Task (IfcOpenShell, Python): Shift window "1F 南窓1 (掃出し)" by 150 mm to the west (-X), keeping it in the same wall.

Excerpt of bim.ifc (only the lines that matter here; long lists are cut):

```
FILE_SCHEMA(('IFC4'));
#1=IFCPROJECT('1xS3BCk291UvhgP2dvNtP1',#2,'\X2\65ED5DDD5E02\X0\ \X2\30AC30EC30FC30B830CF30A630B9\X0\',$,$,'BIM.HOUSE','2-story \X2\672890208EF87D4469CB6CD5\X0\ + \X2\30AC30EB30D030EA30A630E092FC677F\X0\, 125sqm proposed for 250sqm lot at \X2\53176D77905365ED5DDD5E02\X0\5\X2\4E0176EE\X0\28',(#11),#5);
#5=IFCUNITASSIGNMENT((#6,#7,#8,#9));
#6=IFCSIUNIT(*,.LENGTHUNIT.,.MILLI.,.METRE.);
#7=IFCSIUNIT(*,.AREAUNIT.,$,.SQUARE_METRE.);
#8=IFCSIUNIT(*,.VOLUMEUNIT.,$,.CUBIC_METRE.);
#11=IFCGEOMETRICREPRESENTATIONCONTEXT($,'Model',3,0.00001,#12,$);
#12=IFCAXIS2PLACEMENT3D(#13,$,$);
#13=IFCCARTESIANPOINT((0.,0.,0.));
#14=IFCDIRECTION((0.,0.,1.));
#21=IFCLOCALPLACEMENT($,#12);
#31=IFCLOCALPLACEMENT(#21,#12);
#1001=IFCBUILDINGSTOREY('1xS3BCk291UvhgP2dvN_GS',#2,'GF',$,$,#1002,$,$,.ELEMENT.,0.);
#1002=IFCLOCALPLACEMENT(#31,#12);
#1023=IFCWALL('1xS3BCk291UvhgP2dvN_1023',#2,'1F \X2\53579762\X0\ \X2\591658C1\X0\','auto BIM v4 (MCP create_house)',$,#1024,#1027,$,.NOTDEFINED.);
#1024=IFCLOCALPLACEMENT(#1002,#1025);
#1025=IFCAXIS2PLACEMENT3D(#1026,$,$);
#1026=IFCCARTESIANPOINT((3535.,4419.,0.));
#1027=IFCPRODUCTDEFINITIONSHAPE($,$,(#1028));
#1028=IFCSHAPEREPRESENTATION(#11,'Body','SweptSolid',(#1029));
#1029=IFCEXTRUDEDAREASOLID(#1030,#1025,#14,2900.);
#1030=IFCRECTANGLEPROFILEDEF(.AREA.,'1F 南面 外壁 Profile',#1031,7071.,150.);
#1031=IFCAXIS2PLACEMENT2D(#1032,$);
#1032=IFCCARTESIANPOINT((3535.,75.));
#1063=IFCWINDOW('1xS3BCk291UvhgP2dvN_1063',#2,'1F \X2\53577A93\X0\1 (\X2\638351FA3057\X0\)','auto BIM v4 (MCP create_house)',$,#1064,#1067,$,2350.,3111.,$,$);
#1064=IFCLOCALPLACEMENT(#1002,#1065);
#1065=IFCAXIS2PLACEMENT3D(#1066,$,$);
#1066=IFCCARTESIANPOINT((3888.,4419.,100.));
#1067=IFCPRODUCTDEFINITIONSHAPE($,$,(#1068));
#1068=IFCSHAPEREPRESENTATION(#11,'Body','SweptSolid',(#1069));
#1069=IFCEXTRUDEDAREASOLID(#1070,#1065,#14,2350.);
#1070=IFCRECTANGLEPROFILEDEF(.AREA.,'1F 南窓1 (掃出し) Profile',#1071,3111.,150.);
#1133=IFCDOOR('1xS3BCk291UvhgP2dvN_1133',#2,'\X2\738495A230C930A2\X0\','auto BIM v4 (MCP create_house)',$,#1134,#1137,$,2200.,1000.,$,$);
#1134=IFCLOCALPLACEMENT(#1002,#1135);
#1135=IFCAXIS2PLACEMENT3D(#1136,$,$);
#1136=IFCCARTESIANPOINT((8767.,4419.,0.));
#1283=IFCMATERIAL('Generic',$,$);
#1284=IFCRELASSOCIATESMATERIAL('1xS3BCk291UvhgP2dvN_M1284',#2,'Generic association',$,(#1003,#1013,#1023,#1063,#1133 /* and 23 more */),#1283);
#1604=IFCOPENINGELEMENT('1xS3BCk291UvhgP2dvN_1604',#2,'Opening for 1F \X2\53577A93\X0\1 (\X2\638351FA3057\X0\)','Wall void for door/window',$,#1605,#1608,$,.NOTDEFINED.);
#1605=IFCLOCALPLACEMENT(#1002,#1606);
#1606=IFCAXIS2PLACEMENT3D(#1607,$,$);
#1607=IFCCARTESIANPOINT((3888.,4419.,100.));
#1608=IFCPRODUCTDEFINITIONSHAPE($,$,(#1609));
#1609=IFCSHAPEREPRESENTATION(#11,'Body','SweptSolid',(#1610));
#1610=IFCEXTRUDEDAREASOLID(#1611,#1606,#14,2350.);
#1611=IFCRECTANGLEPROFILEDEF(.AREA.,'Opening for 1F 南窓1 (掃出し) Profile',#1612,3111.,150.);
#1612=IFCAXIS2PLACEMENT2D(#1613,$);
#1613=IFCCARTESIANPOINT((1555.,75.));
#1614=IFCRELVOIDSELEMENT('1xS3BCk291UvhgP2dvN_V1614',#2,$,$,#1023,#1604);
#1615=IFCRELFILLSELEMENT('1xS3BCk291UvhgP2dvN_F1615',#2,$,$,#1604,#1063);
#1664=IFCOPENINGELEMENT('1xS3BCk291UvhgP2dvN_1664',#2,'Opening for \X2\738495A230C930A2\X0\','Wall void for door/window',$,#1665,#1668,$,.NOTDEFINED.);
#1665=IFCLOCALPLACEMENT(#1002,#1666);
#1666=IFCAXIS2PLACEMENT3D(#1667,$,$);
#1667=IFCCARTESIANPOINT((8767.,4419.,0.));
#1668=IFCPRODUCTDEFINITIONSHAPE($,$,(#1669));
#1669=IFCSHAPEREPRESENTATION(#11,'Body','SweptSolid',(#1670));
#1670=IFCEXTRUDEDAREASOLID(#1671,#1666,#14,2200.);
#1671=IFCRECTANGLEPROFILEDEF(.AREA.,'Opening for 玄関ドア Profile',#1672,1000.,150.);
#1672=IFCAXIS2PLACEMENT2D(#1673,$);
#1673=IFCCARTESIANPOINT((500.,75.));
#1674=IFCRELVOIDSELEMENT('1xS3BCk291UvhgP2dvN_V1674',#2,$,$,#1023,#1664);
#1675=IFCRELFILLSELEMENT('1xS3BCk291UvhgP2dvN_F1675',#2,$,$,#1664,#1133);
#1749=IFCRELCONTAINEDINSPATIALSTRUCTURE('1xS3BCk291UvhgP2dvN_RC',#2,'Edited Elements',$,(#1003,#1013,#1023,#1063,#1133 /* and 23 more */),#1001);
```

```python
import ifcopenshell
import ifcopenshell.api.geometry
import ifcopenshell.util.placement

model = ifcopenshell.open("bim.ifc")

window = model.by_guid("1xS3BCk291UvhgP2dvN_1063")
opening = window.FillsVoids[0].RelatingOpeningElement
wall = opening.VoidsElements[0].RelatingBuildingElement

wall_matrix = ifcopenshell.util.placement.get_local_placement(wall.ObjectPlacement)
shift = wall_matrix[:3, 0] * -150.0
before = ifcopenshell.util.placement.get_local_placement(window.ObjectPlacement)[:3, 3].copy()

# The window is not placed relative to its opening, so move both.
for product in (opening, window):
    matrix = ifcopenshell.util.placement.get_local_placement(product.ObjectPlacement)
    matrix[:3, 3] += shift
    ifcopenshell.api.geometry.edit_object_placement(model, product=product, matrix=matrix, is_si=False)

after = ifcopenshell.util.placement.get_local_placement(window.ObjectPlacement)[:3, 3]
print("window moved by", (after - before).round(3) + 0.0)

model.write("bim-out.ifc")
```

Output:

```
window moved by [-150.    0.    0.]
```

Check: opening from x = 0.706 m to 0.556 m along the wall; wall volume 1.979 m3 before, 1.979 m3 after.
